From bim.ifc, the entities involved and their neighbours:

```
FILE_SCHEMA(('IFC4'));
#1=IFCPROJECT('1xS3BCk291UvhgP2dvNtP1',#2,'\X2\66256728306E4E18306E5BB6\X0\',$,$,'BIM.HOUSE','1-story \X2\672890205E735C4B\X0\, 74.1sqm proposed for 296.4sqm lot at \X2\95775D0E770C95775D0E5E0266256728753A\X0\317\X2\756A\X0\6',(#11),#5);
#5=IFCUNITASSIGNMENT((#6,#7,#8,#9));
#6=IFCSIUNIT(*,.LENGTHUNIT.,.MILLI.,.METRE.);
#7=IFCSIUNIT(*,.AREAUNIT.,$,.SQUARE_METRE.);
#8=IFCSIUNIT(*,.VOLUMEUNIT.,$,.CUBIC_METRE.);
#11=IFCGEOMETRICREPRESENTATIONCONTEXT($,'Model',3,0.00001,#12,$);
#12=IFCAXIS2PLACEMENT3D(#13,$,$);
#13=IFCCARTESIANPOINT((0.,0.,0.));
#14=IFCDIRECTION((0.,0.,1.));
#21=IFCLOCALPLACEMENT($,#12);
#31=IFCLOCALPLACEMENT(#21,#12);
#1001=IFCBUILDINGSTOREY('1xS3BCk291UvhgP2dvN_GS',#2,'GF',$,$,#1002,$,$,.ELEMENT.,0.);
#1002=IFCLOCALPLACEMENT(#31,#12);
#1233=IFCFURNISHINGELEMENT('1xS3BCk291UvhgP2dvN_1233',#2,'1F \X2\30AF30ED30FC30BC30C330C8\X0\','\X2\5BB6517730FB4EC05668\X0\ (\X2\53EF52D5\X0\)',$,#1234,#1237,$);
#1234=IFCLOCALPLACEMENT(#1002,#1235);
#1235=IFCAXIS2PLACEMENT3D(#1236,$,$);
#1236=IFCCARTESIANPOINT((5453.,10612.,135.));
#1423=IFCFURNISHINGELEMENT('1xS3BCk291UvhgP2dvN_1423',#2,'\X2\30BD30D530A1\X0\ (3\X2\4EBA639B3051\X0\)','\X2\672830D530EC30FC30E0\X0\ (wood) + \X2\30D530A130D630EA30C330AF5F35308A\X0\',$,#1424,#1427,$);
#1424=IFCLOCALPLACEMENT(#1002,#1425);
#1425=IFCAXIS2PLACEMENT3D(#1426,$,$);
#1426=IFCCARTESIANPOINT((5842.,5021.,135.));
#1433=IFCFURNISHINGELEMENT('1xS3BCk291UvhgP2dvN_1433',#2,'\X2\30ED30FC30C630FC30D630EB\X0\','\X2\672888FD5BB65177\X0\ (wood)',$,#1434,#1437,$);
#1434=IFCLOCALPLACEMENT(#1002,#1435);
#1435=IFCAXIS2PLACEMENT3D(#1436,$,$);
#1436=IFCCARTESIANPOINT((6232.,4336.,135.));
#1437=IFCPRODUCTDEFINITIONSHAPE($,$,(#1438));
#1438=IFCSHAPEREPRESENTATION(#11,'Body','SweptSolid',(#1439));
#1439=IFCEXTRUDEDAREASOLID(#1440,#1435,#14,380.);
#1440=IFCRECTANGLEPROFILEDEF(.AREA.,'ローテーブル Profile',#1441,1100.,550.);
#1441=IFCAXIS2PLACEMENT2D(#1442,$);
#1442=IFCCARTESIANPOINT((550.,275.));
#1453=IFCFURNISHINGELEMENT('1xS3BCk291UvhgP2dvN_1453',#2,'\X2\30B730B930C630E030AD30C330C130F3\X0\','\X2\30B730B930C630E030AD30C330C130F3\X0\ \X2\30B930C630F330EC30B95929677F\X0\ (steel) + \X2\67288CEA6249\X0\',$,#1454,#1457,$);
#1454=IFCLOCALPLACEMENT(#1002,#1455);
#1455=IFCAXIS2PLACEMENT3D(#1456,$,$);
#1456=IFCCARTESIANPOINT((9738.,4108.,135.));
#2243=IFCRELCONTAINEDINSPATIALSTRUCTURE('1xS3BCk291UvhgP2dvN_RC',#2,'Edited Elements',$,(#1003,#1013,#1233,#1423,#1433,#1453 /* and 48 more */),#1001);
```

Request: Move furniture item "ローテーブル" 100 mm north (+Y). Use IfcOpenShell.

```python
import ifcopenshell
import ifcopenshell.api.geometry
import ifcopenshell.util.placement
import ifcopenshell.util.unit

model = ifcopenshell.open("bim.ifc")
unit_scale = ifcopenshell.util.unit.calculate_unit_scale(model)

item = model.by_guid("1xS3BCk291UvhgP2dvN_1433")
matrix = ifcopenshell.util.placement.get_local_placement(item.ObjectPlacement)
matrix[1, 3] += 0.1 / unit_scale
ifcopenshell.api.geometry.edit_object_placement(model, product=item, matrix=matrix, is_si=False)

print(ifcopenshell.util.placement.get_local_placement(item.ObjectPlacement).round(3) + 0.0)

model.write("bim_updated.ifc")
```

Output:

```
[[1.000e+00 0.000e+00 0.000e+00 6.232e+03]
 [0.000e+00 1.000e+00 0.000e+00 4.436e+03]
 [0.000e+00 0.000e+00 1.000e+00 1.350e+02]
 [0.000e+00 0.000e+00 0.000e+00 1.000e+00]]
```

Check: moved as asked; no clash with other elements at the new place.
